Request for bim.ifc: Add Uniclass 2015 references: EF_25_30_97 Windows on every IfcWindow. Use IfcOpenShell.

First a look at what the model holds.

```python
import ifcopenshell

model = ifcopenshell.open("bim.ifc")
print(model.schema)
print("classifications:", [c.Name for c in model.by_type("IfcClassification")])
for ifc_class in ("IfcDoor", "IfcRoof", "IfcStair", "IfcWall", "IfcWindow"):
    print(ifc_class, len(model.by_type(ifc_class)))
```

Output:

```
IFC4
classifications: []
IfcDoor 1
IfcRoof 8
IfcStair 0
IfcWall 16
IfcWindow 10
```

```python
import ifcopenshell
import ifcopenshell.api.classification

model = ifcopenshell.open("bim.ifc")

system = ifcopenshell.api.classification.add_classification(model, classification="Uniclass 2015")

codes = {
    "IfcWindow": ("EF_25_30_97", "Windows"),
}
for ifc_class, (code, name) in codes.items():
    products = model.by_type(ifc_class)
    ifcopenshell.api.classification.add_reference(
        model, products=products, classification=system, identification=code, name=name
    )
    print(code, len(products))

model.write("bim_rev.ifc")
```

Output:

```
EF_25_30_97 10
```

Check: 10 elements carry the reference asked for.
